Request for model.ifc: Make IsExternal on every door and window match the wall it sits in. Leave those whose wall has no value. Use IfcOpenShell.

First a look at what the model holds.

```python
import ifcopenshell
import ifcopenshell.util.element

model = ifcopenshell.open("model.ifc")
print(model.schema)
seen = {}
for e in model.by_type("IfcDoor") + model.by_type("IfcWindow"):
    if not e.FillsVoids:
        continue
    host = e.FillsVoids[0].RelatingOpeningElement.VoidsElements[0].RelatingBuildingElement
    own = ifcopenshell.util.element.get_pset(e, f"Pset_{e.is_a()[3:].removesuffix('StandardCase')}Common", "IsExternal")
    wall = ifcopenshell.util.element.get_pset(host, "Pset_WallCommon", "IsExternal")
    seen[e.is_a(), own, wall] = seen.get((e.is_a(), own, wall), 0) + 1
for (cls, own, wall), count in sorted(seen.items(), key=str):
    print(count, cls, "IsExternal:", own, "| host wall:", wall)
```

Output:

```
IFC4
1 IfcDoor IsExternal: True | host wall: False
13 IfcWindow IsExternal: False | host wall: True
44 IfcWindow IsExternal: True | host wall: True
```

```python
import ifcopenshell
import ifcopenshell.api.pset
import ifcopenshell.util.element

model = ifcopenshell.open("model.ifc")

count = 0
for ifc_class, pset_name in (("IfcDoor", "Pset_DoorCommon"), ("IfcWindow", "Pset_WindowCommon")):
    for e in model.by_type(ifc_class):
        if not e.FillsVoids:
            continue
        host = e.FillsVoids[0].RelatingOpeningElement.VoidsElements[0].RelatingBuildingElement
        external = ifcopenshell.util.element.get_pset(host, "Pset_WallCommon", "IsExternal")
        if external is None or ifcopenshell.util.element.get_pset(e, pset_name, "IsExternal") == external:
            continue
        pset = ifcopenshell.api.pset.add_pset(model, product=e, name=pset_name)
        ifcopenshell.api.pset.edit_pset(model, pset=pset, properties={"IsExternal": external})
        count += 1

print(count, "updated")

model.write("model_v2.ifc")
```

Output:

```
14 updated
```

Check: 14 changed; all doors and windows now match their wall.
